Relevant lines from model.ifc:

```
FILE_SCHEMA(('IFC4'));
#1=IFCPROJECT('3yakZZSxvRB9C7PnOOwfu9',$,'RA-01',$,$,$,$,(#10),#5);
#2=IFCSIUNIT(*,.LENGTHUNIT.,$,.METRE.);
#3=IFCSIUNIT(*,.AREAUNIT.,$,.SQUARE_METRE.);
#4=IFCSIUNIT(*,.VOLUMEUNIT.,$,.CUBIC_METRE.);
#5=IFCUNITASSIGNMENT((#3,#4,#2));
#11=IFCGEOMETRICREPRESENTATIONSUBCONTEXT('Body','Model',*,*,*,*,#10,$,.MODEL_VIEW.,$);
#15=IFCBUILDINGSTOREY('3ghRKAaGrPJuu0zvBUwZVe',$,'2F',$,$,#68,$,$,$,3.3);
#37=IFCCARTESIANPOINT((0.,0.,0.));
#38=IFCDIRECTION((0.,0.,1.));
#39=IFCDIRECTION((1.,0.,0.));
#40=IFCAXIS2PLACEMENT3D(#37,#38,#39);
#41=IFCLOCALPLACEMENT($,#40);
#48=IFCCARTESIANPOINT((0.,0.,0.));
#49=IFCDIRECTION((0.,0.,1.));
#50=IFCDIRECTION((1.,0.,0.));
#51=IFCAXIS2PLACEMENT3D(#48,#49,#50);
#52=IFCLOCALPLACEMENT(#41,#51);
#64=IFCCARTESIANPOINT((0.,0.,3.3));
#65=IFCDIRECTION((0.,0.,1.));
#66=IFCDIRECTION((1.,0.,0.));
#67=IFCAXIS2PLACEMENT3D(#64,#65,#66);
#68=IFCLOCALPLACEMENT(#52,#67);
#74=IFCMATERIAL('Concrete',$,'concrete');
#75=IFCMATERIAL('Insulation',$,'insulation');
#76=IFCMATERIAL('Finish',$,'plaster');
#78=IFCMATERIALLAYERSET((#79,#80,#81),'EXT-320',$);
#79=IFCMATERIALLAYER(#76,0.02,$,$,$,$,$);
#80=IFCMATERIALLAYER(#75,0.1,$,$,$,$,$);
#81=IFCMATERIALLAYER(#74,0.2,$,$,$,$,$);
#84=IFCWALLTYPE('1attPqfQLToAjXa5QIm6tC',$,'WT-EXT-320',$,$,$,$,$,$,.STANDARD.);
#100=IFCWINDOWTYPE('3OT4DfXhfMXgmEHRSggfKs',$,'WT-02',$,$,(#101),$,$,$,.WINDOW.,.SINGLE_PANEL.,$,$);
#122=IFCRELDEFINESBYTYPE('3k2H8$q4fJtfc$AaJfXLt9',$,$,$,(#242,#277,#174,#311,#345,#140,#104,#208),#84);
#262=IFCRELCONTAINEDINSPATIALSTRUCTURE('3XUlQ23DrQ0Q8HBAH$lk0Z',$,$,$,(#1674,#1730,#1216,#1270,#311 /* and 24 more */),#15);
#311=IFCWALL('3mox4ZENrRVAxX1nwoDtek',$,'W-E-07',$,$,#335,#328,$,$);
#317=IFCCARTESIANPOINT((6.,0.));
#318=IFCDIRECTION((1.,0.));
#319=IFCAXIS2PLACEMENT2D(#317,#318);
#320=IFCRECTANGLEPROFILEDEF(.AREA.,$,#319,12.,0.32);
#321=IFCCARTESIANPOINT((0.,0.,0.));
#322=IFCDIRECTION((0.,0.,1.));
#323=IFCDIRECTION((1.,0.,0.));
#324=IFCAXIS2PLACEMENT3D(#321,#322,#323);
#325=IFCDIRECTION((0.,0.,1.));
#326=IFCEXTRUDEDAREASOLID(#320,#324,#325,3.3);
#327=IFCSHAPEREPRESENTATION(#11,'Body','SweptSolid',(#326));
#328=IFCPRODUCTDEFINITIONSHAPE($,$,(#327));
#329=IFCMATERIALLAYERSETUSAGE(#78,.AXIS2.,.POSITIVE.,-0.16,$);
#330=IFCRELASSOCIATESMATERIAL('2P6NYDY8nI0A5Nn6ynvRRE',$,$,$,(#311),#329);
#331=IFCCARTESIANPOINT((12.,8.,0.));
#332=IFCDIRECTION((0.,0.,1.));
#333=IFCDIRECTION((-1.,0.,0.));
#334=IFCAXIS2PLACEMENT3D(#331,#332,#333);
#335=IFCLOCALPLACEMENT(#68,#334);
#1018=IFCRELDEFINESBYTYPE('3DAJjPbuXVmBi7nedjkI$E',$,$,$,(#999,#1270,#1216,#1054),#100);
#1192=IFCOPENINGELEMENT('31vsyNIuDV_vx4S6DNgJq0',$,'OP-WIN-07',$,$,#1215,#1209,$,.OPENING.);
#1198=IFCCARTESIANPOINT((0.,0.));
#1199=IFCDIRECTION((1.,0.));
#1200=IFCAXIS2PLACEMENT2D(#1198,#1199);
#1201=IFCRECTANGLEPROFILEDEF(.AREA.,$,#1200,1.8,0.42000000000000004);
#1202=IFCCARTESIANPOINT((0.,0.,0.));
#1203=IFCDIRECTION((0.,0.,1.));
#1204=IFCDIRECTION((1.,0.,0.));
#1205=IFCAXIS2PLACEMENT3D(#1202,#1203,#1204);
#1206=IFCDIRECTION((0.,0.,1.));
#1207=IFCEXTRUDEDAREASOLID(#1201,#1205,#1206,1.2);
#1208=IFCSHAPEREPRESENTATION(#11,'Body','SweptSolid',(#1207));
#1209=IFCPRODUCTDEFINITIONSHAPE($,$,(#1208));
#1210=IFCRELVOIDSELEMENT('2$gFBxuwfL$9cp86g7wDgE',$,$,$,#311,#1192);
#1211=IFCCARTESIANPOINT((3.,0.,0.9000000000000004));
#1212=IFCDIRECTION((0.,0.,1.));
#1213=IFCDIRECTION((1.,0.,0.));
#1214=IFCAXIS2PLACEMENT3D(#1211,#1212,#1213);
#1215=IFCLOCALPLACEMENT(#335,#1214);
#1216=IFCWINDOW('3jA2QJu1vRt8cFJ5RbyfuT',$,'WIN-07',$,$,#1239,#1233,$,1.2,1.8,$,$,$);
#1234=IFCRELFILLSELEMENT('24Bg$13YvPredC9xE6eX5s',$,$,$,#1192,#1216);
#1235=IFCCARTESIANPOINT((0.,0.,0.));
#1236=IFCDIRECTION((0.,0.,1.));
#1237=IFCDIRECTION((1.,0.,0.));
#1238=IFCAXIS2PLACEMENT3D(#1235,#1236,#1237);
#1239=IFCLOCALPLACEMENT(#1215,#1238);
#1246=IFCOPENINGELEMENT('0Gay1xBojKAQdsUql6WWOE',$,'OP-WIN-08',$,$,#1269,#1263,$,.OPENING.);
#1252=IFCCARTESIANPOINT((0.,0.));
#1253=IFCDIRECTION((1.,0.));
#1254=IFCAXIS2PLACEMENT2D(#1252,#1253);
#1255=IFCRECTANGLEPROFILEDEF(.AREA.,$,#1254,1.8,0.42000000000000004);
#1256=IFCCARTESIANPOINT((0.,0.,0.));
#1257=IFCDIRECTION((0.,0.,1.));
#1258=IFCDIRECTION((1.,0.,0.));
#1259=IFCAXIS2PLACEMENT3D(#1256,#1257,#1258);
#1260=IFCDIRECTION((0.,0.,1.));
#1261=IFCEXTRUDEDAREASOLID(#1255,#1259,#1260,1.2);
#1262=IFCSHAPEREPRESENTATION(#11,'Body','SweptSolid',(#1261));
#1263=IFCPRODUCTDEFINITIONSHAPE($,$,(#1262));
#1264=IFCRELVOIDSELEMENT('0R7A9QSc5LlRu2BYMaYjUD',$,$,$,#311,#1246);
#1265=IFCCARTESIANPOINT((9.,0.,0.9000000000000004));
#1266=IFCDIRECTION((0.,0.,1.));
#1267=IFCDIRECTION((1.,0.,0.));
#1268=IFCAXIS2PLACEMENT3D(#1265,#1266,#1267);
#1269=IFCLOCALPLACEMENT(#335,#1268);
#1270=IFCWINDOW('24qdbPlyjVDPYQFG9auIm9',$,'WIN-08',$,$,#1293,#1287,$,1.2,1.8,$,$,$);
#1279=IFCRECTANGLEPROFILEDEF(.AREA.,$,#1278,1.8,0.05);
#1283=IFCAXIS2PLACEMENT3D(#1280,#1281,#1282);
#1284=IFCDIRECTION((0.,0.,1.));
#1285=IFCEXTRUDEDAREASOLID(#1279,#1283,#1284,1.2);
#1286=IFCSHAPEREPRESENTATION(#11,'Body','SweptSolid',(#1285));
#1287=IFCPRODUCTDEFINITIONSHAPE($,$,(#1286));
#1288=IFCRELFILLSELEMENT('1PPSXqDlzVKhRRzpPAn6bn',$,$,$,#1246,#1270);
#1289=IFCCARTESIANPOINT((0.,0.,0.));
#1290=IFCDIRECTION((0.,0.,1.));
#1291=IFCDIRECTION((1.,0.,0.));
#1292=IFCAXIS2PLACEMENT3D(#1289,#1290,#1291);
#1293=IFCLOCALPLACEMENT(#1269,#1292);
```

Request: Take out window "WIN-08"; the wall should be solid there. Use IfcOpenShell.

```python
import ifcopenshell
import ifcopenshell.api.feature
import ifcopenshell.api.root
import ifcopenshell.geom
import ifcopenshell.util.shape

model = ifcopenshell.open("model.ifc")
settings = ifcopenshell.geom.settings()


def volume(element):
    """Net volume in cubic metres, openings subtracted."""
    shape = ifcopenshell.geom.create_shape(settings, element)
    return ifcopenshell.util.shape.get_volume(shape.geometry)


window = model.by_id(1270)
opening = window.FillsVoids[0].RelatingOpeningElement
wall = opening.VoidsElements[0].RelatingBuildingElement
before = volume(wall)

ifcopenshell.api.root.remove_product(model, product=window)
ifcopenshell.api.feature.remove_feature(model, feature=opening)

after = volume(wall)

print(f"wall volume {before:.3f} -> {after:.3f} m3")

model.write("model_v2.ifc")
```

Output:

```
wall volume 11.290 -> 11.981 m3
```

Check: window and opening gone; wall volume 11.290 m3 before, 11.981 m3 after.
